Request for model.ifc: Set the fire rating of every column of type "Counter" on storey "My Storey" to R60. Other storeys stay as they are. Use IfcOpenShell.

First a look at what the model holds.

```python
import ifcopenshell
import ifcopenshell.util.element

model = ifcopenshell.open("model.ifc")
print(model.schema)
storey = next(s for s in model.by_type("IfcBuildingStorey") if s.Name == "My Storey")
columns = [e for e in ifcopenshell.util.element.get_decomposition(storey) if e.is_a("IfcColumn")]
seen = {}
for e in columns:
    element_type = ifcopenshell.util.element.get_type(e)
    key = (element_type.Name if element_type != e and element_type else None, ifcopenshell.util.element.get_pset(e, "Pset_ColumnCommon", "FireRating"))
    seen[key] = seen.get(key, 0) + 1
for (name, value), count in sorted(seen.items(), key=str):
    print(count, "x", name, "|", value)
```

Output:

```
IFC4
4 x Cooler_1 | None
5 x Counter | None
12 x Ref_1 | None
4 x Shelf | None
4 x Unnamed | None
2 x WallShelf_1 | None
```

```python
import ifcopenshell
import ifcopenshell.api.pset
import ifcopenshell.util.element

model = ifcopenshell.open("model.ifc")

storey = next(s for s in model.by_type("IfcBuildingStorey") if s.Name == "My Storey")
columns = [e for e in ifcopenshell.util.element.get_decomposition(storey) if e.is_a("IfcColumn")]

count = 0
for e in columns:
    element_type = ifcopenshell.util.element.get_type(e)
    if element_type in (None, e) or element_type.Name != "Counter":
        continue
    # add_pset returns the element's existing set when there is one.
    pset = ifcopenshell.api.pset.add_pset(model, product=e, name="Pset_ColumnCommon")
    ifcopenshell.api.pset.edit_pset(model, pset=pset, properties={"FireRating": "R60"})
    count += 1

print(count, "columns updated")

model.write("model_rev.ifc")
```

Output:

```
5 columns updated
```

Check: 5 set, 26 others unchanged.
